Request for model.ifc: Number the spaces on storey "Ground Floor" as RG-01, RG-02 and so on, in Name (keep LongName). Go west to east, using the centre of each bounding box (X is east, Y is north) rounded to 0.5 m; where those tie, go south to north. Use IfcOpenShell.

First a look at what the model holds.

```python
import ifcopenshell
import ifcopenshell.util.element
import ifcopenshell.util.placement

model = ifcopenshell.open("model.ifc")
print(model.schema)
storey = next(s for s in model.by_type("IfcBuildingStorey") if s.Name == "Ground Floor")
spaces = [e for e in ifcopenshell.util.element.get_decomposition(storey) if e.is_a("IfcSpace")]
for e in sorted(spaces, key=lambda e: e.id()):
    origin = ifcopenshell.util.placement.get_local_placement(e.ObjectPlacement)[:3, 3]
    print(e.id(), e.Name, e.LongName, origin.round(2) + 0.0, sep=" | ")
```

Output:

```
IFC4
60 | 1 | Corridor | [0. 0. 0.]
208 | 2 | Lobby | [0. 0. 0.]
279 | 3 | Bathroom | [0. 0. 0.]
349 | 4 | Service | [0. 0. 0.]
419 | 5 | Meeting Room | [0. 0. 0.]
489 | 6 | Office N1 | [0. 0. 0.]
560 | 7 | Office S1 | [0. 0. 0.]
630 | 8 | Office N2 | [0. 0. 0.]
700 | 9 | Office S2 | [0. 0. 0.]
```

```python
import ifcopenshell
import ifcopenshell.geom
import ifcopenshell.util.element
import ifcopenshell.util.shape

model = ifcopenshell.open("model.ifc")
settings = ifcopenshell.geom.settings()
settings.set("use-world-coords", True)


def centre(element):
    shape = ifcopenshell.geom.create_shape(settings, element)
    return ifcopenshell.util.shape.get_bbox_centroid(shape.geometry)


storey = next(s for s in model.by_type("IfcBuildingStorey") if s.Name == "Ground Floor")
spaces = [e for e in ifcopenshell.util.element.get_decomposition(storey) if e.is_a("IfcSpace")]

# Insertion points can sit at a corner or the storey origin, so sort by the geometry (in metres).
centres = {e: centre(e) for e in spaces}
spaces.sort(key=lambda e: (round(centres[e][0] / 0.5), centres[e][1]))

for i, e in enumerate(spaces, start=1):
    number = f"RG-{i:02d}"
    e.Name = number
    print(e.id(), number)

model.write("model_rev.ifc")
```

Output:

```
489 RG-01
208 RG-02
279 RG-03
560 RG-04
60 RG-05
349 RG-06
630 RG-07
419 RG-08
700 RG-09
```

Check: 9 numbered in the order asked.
